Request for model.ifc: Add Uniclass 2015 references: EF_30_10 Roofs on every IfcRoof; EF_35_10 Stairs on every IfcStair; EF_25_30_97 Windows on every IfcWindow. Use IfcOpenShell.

First a look at what the model holds.

```python
import ifcopenshell

model = ifcopenshell.open("model.ifc")
print(model.schema)
print("classifications:", [c.Name for c in model.by_type("IfcClassification")])
for ifc_class in ("IfcDoor", "IfcRoof", "IfcStair", "IfcWall", "IfcWindow"):
    print(ifc_class, len(model.by_type(ifc_class)))
```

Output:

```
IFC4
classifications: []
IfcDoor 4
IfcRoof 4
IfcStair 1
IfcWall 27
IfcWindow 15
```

```python
import ifcopenshell
import ifcopenshell.api.classification

model = ifcopenshell.open("model.ifc")

system = ifcopenshell.api.classification.add_classification(model, classification="Uniclass 2015")

codes = {
    "IfcRoof": ("EF_30_10", "Roofs"),
    "IfcStair": ("EF_35_10", "Stairs"),
    "IfcWindow": ("EF_25_30_97", "Windows"),
}
for ifc_class, (code, name) in codes.items():
    products = model.by_type(ifc_class)
    ifcopenshell.api.classification.add_reference(
        model, products=products, classification=system, identification=code, name=name
    )
    print(code, len(products))

model.write("model_updated.ifc")
```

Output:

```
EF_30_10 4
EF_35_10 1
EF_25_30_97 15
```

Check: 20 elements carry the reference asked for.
